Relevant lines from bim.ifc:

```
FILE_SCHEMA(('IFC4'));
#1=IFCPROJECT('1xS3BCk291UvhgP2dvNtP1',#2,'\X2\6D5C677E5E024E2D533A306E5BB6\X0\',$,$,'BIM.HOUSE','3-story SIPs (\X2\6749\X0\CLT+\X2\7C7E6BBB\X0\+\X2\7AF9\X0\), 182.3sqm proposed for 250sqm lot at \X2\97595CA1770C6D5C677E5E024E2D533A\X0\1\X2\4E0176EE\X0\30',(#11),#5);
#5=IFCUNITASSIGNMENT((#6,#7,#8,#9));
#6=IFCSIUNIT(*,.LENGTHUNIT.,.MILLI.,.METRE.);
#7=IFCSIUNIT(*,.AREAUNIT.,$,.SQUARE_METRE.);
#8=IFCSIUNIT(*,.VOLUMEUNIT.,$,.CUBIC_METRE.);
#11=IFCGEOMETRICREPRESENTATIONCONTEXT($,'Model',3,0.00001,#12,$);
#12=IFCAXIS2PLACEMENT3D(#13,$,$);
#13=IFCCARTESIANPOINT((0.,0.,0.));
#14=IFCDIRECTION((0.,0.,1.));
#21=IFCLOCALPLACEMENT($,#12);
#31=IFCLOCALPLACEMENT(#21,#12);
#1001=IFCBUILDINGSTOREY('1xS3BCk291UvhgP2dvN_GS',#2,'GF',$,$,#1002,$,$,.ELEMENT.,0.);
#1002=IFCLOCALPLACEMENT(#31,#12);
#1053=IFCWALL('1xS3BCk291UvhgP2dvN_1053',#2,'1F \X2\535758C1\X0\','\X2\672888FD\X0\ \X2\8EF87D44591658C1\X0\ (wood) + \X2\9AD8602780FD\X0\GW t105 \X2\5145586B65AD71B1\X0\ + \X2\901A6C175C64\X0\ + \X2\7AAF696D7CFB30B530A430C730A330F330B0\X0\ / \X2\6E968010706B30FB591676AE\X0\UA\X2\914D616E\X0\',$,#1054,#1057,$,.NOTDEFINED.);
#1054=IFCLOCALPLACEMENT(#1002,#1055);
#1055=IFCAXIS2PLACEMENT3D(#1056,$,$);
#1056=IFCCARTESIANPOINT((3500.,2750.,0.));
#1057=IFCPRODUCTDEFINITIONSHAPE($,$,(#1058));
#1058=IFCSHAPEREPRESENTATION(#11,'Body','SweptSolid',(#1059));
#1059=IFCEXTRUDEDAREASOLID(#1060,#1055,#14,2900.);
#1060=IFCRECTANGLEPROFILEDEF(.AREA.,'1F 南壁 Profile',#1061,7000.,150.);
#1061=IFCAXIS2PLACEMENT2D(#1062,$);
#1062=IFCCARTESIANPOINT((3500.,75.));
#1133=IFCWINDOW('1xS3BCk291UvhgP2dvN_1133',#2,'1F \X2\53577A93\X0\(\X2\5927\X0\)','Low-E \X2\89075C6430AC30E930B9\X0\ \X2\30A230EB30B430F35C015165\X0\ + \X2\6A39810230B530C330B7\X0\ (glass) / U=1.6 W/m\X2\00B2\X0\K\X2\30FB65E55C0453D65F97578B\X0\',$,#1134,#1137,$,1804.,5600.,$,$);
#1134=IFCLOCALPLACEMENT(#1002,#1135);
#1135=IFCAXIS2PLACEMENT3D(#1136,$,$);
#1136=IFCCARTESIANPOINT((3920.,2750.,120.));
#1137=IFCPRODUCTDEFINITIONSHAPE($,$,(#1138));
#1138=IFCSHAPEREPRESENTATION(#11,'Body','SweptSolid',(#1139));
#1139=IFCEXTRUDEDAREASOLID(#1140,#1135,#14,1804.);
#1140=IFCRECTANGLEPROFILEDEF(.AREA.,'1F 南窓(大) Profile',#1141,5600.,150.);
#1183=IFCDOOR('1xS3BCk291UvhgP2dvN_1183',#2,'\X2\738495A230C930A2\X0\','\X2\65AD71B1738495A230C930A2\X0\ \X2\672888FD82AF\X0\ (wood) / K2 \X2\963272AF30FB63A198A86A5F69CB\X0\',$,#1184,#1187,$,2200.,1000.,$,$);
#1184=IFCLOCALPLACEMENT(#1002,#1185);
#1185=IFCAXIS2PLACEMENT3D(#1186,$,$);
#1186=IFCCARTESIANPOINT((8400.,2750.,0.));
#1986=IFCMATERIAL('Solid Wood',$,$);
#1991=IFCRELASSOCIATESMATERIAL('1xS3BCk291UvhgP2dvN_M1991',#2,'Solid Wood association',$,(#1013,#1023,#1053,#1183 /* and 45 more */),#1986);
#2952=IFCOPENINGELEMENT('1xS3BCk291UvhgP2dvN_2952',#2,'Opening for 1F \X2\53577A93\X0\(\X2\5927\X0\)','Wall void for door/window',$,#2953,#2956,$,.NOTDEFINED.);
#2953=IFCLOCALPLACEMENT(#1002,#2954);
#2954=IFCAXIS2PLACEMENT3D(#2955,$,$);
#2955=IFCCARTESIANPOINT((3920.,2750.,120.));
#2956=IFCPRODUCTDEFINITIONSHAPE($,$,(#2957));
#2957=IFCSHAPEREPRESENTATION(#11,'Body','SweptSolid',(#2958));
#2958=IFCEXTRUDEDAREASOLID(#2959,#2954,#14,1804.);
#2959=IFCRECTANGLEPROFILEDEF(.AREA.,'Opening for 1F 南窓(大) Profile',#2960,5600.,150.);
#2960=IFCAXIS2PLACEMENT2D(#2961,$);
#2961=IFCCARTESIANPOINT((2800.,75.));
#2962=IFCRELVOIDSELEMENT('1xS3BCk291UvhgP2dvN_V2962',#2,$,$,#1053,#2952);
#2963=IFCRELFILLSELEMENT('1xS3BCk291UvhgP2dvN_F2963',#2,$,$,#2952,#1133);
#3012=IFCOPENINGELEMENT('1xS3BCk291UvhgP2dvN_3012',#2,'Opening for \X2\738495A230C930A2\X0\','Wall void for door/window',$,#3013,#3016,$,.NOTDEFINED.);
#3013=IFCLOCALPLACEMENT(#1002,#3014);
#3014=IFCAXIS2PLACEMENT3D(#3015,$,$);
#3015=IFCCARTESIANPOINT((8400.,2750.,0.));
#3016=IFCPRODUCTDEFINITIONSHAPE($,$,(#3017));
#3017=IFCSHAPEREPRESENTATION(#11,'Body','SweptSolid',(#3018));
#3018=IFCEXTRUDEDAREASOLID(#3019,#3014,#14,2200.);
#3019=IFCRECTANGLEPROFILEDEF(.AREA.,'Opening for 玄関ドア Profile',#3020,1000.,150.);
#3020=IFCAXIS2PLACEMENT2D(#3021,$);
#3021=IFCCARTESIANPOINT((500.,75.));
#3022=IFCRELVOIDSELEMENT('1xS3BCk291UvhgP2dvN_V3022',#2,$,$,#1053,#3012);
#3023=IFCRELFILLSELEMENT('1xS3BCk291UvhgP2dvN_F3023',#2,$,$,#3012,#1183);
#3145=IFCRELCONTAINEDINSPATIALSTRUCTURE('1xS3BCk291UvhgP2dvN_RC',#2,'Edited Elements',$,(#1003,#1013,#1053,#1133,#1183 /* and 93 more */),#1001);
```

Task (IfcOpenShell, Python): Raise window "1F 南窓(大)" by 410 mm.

```python
import numpy as np
import ifcopenshell
import ifcopenshell.api.geometry
import ifcopenshell.util.placement
import ifcopenshell.util.unit

model = ifcopenshell.open("bim.ifc")
unit_scale = ifcopenshell.util.unit.calculate_unit_scale(model)

window = model.by_id(1133)
opening = window.FillsVoids[0].RelatingOpeningElement
dz = 0.41 / unit_scale

shift = np.array([0.0, 0.0, dz])
# The window is not placed relative to its opening, so move both.
for product in (opening, window):
    matrix = ifcopenshell.util.placement.get_local_placement(product.ObjectPlacement)
    matrix[:3, 3] += shift
    ifcopenshell.api.geometry.edit_object_placement(model, product=product, matrix=matrix, is_si=False)

print(f"moved by {dz * unit_scale:+.3f} m")

model.write("bim_edited.ifc")
```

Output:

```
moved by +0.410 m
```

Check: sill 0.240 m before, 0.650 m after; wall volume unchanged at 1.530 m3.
